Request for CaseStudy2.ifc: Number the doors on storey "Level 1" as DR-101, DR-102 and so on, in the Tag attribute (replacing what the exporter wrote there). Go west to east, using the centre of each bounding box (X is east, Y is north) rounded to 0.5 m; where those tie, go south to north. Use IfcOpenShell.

First a look at what the model holds.

```python
import ifcopenshell
import ifcopenshell.util.element
import ifcopenshell.util.placement

model = ifcopenshell.open("CaseStudy2.ifc")
print(model.schema)
storey = next(s for s in model.by_type("IfcBuildingStorey") if s.Name == "Level 1")
doors = [e for e in ifcopenshell.util.element.get_decomposition(storey) if e.is_a("IfcDoor")]
for e in sorted(doors, key=lambda e: e.id()):
    origin = ifcopenshell.util.placement.get_local_placement(e.ObjectPlacement)[:3, 3]
    print(e.id(), e.Tag, e.Name, origin.round(2) + 0.0, sep=" | ")
```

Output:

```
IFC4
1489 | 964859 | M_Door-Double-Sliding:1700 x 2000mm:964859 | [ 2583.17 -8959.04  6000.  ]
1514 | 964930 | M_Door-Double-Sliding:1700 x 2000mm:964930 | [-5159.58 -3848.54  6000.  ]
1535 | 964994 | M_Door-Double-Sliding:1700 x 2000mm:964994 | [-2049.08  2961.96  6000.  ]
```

```python
import ifcopenshell
import ifcopenshell.geom
import ifcopenshell.util.element
import ifcopenshell.util.shape

model = ifcopenshell.open("CaseStudy2.ifc")
settings = ifcopenshell.geom.settings()
settings.set("use-world-coords", True)


def centre(element):
    shape = ifcopenshell.geom.create_shape(settings, element)
    return ifcopenshell.util.shape.get_bbox_centroid(shape.geometry)


storey = next(s for s in model.by_type("IfcBuildingStorey") if s.Name == "Level 1")
doors = [e for e in ifcopenshell.util.element.get_decomposition(storey) if e.is_a("IfcDoor")]

# Insertion points can sit at a corner or the storey origin, so sort by the geometry (in metres).
centres = {e: centre(e) for e in doors}
doors.sort(key=lambda e: (round(centres[e][0] / 0.5), centres[e][1]))

for i, e in enumerate(doors, start=1):
    number = f"DR-1{i:02d}"
    e.Tag = number
    print(e.id(), number)

model.write("CaseStudy2_updated.ifc")
```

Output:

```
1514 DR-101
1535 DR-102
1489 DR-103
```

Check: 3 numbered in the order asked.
